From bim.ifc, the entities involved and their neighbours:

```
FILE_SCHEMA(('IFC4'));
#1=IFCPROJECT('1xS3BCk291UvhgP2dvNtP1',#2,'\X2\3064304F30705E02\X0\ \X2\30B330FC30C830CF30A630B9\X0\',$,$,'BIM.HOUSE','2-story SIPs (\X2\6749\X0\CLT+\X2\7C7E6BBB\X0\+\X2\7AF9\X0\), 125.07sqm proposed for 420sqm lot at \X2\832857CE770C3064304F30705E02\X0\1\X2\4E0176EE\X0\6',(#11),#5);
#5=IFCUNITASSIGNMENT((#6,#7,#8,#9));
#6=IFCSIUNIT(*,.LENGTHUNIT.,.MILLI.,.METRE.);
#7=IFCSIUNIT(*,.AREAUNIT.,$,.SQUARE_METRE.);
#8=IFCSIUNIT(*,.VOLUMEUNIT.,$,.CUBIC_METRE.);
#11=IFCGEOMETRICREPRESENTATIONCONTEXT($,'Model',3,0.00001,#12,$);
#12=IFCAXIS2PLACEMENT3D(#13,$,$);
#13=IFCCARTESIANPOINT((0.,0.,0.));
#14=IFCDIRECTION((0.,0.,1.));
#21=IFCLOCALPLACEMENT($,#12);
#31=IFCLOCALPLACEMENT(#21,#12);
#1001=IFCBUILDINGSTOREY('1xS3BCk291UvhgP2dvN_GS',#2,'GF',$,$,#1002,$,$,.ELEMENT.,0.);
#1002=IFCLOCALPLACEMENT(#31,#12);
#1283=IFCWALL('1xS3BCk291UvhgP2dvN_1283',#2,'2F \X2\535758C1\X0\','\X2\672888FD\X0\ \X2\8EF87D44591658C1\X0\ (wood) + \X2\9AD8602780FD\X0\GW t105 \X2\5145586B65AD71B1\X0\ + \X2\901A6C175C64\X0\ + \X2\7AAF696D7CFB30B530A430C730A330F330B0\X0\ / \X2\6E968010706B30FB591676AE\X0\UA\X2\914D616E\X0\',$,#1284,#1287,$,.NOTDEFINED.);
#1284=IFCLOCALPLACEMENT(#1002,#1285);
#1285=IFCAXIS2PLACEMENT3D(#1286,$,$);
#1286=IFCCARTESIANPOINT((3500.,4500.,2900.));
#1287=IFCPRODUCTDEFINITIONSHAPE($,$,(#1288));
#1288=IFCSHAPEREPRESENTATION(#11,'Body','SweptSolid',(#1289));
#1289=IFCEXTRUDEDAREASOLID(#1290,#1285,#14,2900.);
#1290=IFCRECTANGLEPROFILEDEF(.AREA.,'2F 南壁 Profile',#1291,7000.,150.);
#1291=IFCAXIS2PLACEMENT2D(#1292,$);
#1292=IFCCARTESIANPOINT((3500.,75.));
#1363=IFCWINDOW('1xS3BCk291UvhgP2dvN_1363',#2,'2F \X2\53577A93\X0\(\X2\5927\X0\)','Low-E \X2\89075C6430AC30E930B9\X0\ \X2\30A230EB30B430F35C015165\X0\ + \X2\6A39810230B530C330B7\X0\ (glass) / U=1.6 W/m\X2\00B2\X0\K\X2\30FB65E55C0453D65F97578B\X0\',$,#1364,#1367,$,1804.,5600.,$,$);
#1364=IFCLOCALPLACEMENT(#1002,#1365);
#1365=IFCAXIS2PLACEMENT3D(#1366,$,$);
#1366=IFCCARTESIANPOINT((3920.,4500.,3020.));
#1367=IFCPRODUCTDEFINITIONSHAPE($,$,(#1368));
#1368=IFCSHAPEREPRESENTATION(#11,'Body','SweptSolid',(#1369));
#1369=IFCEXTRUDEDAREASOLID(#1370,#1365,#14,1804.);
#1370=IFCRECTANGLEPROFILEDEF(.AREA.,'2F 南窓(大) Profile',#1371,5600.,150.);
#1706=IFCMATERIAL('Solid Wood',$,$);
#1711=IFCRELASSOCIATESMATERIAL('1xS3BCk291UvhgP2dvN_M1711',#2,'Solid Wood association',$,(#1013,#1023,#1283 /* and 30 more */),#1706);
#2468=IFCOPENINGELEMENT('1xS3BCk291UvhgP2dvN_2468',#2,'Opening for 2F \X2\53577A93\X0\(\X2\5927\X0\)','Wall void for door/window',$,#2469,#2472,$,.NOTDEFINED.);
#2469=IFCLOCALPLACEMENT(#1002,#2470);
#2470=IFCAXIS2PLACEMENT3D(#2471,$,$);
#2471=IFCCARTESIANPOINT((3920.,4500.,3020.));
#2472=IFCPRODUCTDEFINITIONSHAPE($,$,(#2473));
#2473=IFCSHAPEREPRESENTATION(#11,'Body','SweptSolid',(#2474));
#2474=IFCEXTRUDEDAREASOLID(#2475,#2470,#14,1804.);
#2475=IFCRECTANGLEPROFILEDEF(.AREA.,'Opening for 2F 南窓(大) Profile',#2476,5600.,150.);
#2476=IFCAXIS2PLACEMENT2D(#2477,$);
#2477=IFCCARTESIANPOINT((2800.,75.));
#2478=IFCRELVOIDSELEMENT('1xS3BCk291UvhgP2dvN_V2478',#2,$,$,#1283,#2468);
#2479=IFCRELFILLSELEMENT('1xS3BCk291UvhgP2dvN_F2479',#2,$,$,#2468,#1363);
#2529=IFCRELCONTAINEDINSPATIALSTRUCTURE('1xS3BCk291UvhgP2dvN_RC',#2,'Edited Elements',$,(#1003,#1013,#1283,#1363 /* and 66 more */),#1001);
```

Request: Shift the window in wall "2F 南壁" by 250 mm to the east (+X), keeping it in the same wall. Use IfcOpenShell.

```python
import ifcopenshell
import ifcopenshell.api.geometry
import ifcopenshell.util.placement
import ifcopenshell.util.unit

model = ifcopenshell.open("bim.ifc")
unit_scale = ifcopenshell.util.unit.calculate_unit_scale(model)

window = model.by_id(1363)
opening = window.FillsVoids[0].RelatingOpeningElement
wall = opening.VoidsElements[0].RelatingBuildingElement

wall_matrix = ifcopenshell.util.placement.get_local_placement(wall.ObjectPlacement)
shift = wall_matrix[:3, 0] * 0.25 / unit_scale
before = ifcopenshell.util.placement.get_local_placement(window.ObjectPlacement)[:3, 3].copy()

# The window is not placed relative to its opening, so move both.
for product in (opening, window):
    matrix = ifcopenshell.util.placement.get_local_placement(product.ObjectPlacement)
    matrix[:3, 3] += shift
    ifcopenshell.api.geometry.edit_object_placement(model, product=product, matrix=matrix, is_si=False)

after = ifcopenshell.util.placement.get_local_placement(window.ObjectPlacement)[:3, 3]
print("window moved by", (after - before).round(3) + 0.0)

model.write("bim-out.ifc")
```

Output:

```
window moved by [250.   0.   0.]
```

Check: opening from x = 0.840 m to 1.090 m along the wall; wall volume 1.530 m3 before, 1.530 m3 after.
